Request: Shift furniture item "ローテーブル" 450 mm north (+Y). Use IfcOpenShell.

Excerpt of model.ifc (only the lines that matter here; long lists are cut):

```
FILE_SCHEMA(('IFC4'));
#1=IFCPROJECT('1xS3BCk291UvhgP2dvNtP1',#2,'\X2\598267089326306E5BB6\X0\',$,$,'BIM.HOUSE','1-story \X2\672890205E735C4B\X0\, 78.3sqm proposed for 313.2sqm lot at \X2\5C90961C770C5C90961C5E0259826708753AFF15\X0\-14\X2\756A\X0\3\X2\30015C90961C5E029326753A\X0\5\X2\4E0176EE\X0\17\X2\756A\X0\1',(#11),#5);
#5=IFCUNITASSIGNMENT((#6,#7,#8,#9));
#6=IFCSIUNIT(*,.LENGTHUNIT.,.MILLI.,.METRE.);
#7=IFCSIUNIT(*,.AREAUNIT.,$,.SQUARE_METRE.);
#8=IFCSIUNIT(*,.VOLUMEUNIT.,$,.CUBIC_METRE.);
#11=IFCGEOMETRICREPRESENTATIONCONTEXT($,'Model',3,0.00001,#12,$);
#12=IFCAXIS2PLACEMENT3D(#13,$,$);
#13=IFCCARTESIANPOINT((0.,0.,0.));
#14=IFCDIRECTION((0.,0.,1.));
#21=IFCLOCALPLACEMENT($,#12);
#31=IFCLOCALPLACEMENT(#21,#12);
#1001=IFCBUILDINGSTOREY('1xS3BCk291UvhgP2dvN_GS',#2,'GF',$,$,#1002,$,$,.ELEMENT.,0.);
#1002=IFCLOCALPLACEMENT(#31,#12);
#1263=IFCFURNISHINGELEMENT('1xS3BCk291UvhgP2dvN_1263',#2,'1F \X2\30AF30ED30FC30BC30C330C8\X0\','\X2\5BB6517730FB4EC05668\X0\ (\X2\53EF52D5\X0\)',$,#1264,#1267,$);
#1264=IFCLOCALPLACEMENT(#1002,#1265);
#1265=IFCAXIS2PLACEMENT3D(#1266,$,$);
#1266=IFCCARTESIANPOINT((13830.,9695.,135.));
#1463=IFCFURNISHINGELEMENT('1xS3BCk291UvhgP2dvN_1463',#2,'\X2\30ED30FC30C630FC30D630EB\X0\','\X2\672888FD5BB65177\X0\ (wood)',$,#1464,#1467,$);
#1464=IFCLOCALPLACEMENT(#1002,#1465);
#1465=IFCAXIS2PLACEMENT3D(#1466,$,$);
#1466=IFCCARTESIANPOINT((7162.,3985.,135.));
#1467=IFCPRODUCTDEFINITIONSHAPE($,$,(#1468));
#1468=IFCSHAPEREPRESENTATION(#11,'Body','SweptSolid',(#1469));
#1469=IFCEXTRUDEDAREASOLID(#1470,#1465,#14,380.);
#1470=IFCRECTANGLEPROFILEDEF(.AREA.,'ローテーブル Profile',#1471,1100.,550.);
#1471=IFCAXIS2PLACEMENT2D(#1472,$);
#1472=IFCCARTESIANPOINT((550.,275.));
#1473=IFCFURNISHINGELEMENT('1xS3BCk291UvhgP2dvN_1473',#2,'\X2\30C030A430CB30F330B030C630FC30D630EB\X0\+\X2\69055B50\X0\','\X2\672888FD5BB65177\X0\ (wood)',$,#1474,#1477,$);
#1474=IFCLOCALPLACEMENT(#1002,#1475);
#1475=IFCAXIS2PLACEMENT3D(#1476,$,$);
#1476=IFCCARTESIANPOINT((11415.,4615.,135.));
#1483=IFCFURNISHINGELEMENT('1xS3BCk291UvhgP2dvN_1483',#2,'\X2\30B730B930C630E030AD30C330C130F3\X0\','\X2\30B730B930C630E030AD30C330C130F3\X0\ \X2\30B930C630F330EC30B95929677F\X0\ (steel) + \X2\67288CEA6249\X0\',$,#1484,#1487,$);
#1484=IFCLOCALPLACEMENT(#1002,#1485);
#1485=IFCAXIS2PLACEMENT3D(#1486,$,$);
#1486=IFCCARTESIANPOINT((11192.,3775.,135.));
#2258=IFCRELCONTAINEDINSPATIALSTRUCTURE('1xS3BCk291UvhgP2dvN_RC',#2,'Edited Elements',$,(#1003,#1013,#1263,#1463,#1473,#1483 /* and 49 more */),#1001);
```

```python
import ifcopenshell
import ifcopenshell.api.geometry
import ifcopenshell.util.placement
import ifcopenshell.util.unit

model = ifcopenshell.open("model.ifc")
unit_scale = ifcopenshell.util.unit.calculate_unit_scale(model)

item = model.by_guid("1xS3BCk291UvhgP2dvN_1463")
matrix = ifcopenshell.util.placement.get_local_placement(item.ObjectPlacement)
matrix[1, 3] += 0.45 / unit_scale
ifcopenshell.api.geometry.edit_object_placement(model, product=item, matrix=matrix, is_si=False)

print(ifcopenshell.util.placement.get_local_placement(item.ObjectPlacement).round(3) + 0.0)

model.write("model-out.ifc")
```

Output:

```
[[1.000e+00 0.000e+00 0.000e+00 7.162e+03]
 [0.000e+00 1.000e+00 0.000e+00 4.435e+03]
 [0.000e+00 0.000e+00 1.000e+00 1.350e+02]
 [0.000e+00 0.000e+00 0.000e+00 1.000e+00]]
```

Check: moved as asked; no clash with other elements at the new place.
